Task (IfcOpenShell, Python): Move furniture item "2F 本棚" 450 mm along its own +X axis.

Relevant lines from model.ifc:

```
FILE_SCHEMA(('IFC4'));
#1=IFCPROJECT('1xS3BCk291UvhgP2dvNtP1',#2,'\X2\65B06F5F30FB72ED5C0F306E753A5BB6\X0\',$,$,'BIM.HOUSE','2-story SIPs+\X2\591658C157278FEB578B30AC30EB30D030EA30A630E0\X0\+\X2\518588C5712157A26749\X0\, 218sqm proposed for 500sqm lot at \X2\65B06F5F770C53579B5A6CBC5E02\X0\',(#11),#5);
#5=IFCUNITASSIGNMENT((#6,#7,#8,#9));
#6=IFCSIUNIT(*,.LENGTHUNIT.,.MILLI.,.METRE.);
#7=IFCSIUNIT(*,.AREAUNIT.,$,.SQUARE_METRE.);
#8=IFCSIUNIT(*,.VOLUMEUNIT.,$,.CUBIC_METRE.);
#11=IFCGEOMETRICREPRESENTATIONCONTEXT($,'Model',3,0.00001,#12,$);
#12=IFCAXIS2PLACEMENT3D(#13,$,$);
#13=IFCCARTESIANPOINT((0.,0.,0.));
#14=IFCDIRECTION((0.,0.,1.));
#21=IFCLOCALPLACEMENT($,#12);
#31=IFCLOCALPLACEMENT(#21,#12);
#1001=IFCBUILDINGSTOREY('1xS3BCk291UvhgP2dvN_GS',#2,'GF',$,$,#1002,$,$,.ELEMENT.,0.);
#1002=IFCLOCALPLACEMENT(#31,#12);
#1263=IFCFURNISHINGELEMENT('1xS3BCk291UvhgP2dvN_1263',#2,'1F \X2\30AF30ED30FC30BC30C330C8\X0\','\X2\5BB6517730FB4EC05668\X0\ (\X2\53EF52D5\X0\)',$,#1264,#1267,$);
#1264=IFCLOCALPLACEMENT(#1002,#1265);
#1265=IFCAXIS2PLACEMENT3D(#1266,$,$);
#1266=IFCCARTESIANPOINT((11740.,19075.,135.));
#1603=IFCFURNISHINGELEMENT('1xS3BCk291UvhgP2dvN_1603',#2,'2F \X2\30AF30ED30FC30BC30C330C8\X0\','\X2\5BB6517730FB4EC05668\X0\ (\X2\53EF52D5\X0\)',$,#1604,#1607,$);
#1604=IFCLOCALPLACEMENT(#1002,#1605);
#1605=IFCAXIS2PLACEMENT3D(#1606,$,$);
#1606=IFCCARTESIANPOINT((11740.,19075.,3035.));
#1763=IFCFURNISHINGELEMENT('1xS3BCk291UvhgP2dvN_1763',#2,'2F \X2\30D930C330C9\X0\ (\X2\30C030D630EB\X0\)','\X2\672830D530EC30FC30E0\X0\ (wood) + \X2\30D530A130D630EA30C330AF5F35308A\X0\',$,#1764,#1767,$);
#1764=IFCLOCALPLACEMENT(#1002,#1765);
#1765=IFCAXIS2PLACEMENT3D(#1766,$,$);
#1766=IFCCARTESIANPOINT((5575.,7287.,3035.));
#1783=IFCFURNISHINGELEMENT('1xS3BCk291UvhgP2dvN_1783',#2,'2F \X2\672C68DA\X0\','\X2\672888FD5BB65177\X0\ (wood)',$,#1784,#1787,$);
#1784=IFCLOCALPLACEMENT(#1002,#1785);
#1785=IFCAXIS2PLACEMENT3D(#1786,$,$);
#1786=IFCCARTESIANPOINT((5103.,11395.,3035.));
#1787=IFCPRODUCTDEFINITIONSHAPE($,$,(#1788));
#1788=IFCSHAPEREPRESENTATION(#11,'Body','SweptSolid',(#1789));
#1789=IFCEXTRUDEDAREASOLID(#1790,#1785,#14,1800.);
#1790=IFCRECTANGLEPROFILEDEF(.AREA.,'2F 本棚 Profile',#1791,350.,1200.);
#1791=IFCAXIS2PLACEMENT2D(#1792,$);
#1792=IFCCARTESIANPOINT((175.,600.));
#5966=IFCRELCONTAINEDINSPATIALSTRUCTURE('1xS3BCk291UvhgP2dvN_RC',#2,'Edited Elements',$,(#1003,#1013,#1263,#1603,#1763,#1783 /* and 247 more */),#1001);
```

```python
import ifcopenshell
import ifcopenshell.api.geometry
import ifcopenshell.util.placement

model = ifcopenshell.open("model.ifc")

item = model.by_guid("1xS3BCk291UvhgP2dvN_1783")
matrix = ifcopenshell.util.placement.get_local_placement(item.ObjectPlacement)
matrix[:3, 3] += matrix[:3, 0] * 450.0
ifcopenshell.api.geometry.edit_object_placement(model, product=item, matrix=matrix, is_si=False)

print(ifcopenshell.util.placement.get_local_placement(item.ObjectPlacement).round(3) + 0.0)

model.write("model_edited.ifc")
```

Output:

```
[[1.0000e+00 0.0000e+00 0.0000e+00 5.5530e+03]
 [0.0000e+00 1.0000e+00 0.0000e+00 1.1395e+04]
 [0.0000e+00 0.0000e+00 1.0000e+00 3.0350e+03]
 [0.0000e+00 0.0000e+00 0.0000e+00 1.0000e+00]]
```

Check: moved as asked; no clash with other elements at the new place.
